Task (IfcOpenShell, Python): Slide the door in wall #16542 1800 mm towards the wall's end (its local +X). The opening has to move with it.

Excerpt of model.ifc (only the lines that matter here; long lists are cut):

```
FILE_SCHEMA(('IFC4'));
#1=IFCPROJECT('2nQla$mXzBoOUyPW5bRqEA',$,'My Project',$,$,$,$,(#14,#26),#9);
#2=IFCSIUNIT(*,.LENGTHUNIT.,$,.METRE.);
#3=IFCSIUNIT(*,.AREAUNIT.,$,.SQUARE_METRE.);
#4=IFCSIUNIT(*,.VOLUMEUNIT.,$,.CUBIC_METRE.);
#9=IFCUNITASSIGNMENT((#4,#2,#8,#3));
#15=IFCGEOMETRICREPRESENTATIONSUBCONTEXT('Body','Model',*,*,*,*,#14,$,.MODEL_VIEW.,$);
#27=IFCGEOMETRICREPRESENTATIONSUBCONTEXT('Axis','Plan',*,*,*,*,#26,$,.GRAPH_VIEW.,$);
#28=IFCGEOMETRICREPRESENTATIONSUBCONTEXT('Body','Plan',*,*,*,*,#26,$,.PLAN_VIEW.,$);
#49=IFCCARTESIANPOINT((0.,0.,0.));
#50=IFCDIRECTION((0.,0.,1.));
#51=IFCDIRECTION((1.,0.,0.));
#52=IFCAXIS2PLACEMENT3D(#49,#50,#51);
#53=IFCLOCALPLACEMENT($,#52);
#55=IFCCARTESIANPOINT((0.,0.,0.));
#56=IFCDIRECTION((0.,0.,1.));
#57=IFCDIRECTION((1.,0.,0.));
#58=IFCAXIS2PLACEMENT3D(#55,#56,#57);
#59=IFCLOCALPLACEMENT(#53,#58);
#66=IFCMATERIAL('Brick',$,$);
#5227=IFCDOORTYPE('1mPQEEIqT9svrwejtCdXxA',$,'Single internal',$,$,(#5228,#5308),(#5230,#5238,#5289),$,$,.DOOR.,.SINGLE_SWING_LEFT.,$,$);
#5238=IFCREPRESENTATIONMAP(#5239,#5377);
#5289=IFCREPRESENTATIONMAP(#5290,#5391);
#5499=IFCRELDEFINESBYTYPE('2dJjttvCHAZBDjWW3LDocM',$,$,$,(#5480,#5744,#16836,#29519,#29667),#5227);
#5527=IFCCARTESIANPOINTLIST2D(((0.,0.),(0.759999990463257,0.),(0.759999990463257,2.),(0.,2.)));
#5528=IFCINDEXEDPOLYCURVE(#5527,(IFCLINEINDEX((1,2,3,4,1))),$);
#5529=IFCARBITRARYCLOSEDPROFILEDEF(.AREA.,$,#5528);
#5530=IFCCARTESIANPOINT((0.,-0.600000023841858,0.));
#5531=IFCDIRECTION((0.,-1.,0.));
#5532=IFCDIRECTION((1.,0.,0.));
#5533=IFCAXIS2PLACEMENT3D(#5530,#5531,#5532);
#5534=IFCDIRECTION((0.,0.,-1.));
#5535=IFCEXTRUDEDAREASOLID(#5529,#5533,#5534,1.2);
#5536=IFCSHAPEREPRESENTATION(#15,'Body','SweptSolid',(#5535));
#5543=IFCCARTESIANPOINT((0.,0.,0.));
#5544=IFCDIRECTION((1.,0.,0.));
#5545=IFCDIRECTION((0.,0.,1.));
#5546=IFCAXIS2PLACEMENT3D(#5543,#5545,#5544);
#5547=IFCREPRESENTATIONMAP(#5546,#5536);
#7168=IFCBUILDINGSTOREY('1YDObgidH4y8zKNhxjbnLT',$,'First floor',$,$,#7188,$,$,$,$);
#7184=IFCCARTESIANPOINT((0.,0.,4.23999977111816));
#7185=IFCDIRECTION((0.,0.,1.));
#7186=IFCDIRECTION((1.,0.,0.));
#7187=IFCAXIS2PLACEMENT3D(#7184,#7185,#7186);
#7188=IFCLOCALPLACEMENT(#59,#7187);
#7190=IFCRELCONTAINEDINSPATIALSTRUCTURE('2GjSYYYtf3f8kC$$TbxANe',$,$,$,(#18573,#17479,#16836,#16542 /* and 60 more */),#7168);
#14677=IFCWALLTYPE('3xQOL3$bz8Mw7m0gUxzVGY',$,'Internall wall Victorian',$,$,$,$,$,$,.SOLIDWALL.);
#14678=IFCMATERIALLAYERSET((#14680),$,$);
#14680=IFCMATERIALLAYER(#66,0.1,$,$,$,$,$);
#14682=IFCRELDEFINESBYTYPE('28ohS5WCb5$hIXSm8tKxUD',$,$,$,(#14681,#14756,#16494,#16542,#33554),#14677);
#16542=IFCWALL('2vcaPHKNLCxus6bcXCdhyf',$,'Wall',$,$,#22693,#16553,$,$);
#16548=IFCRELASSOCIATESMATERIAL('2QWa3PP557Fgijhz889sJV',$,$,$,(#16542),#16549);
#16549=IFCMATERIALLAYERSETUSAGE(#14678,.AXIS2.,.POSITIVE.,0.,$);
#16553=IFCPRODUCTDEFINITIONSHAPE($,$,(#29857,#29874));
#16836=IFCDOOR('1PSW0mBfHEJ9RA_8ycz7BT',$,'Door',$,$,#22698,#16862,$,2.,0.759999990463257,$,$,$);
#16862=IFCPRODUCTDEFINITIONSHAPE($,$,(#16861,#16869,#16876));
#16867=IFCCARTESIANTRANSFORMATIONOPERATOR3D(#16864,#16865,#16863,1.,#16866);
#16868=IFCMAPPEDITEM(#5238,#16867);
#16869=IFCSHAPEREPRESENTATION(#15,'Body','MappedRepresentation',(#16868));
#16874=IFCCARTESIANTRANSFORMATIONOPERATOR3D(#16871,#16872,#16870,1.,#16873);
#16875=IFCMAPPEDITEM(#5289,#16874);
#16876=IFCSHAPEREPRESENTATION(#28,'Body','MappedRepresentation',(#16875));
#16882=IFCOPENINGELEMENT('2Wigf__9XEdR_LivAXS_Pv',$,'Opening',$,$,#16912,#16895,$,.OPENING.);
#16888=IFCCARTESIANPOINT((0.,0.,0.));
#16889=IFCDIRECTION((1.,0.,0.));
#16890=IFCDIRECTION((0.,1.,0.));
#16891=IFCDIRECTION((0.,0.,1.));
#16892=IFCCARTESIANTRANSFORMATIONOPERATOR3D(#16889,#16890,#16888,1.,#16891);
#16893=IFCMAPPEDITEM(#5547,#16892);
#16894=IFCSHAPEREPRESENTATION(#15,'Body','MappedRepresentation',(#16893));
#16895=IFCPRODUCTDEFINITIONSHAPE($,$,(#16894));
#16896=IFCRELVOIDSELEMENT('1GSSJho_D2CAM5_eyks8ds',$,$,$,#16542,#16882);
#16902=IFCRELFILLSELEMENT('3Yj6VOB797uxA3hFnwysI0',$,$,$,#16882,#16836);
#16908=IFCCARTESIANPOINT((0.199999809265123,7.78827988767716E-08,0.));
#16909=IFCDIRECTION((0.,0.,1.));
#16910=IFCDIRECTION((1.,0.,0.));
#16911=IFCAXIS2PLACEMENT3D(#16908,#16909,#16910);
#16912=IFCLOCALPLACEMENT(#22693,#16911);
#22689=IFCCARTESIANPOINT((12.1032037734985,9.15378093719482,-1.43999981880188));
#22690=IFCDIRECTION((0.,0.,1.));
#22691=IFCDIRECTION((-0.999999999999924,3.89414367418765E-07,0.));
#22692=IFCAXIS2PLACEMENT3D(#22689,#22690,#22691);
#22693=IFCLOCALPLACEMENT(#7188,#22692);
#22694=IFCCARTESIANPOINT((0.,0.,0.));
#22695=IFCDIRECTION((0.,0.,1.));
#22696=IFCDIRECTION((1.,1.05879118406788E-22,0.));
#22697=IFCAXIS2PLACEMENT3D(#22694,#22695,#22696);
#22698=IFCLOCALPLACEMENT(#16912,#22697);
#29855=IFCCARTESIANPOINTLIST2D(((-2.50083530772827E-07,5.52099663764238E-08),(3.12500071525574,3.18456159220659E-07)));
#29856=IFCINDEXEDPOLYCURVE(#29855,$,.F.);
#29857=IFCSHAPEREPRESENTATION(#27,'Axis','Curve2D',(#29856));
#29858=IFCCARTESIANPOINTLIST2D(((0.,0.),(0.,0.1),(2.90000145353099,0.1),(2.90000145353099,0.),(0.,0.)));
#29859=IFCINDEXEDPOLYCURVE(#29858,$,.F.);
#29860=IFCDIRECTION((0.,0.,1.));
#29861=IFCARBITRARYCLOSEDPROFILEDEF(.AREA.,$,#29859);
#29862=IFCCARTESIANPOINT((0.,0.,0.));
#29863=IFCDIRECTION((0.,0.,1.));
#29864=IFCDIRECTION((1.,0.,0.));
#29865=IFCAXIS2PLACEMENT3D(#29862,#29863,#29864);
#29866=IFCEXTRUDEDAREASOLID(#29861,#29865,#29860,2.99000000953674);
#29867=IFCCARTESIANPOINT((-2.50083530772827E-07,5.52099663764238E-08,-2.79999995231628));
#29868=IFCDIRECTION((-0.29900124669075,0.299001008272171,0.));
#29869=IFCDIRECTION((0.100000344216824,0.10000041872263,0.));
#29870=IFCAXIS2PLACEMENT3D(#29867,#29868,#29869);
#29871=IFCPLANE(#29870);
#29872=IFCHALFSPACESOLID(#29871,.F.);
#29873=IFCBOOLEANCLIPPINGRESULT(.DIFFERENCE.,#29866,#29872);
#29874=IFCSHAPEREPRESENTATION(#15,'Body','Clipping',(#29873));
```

```python
import ifcopenshell
import ifcopenshell.api.geometry
import ifcopenshell.util.placement

model = ifcopenshell.open("model.ifc")

door = model.by_guid("1PSW0mBfHEJ9RA_8ycz7BT")
opening = door.FillsVoids[0].RelatingOpeningElement
wall = opening.VoidsElements[0].RelatingBuildingElement

wall_matrix = ifcopenshell.util.placement.get_local_placement(wall.ObjectPlacement)
shift = wall_matrix[:3, 0] * 1.8
before = ifcopenshell.util.placement.get_local_placement(door.ObjectPlacement)[:3, 3].copy()

# The door is placed relative to its opening, so it follows when the opening moves.
matrix = ifcopenshell.util.placement.get_local_placement(opening.ObjectPlacement)
matrix[:3, 3] += shift
ifcopenshell.api.geometry.edit_object_placement(
    model, product=opening, matrix=matrix, is_si=False, should_transform_children=True
)

after = ifcopenshell.util.placement.get_local_placement(door.ObjectPlacement)[:3, 3]
print("door moved by", (after - before).round(3) + 0.0)

model.write("model_v2.ifc")
```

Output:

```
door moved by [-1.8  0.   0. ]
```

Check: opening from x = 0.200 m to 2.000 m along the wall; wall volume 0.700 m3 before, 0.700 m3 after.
